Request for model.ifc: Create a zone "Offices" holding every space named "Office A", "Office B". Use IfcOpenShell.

First a look at what the model holds.

```python
import ifcopenshell

model = ifcopenshell.open("model.ifc")
print(model.schema)
seen = {}
for space in model.by_type("IfcSpace"):
    seen[space.LongName] = seen.get(space.LongName, 0) + 1
for name, count in sorted(seen.items(), key=str):
    print(count, "x", name)
print("zones:", [z.Name for z in model.by_type("IfcZone")][:20])
```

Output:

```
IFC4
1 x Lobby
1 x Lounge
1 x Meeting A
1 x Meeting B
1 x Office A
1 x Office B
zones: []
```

```python
import ifcopenshell
import ifcopenshell.api.group
import ifcopenshell.api.root

model = ifcopenshell.open("model.ifc")

names = {"Office A", "Office B"}
spaces = [s for s in model.by_type("IfcSpace") if s.LongName in names]

zone = ifcopenshell.api.root.create_entity(model, ifc_class="IfcZone", name="Offices")
ifcopenshell.api.group.assign_group(model, products=spaces, group=zone)
print(len(spaces), "spaces in", zone.Name)

model.write("model_v2.ifc")
```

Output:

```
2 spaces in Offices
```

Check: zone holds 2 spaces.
